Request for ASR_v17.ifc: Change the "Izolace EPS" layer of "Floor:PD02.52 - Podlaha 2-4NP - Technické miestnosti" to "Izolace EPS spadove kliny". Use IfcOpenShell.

First a look at what the model holds.

```python
import ifcopenshell
import ifcopenshell.util.element

model = ifcopenshell.open("ASR_v17.ifc")
print(model.schema)
for layer_set in model.by_type("IfcMaterialLayerSet"):
    if layer_set.LayerSetName == "Floor:PD02.52 - Podlaha 2-4NP - Technické miestnosti":
        for layer in layer_set.MaterialLayers:
            print(layer.id(), layer.Material and layer.Material.Name, layer.LayerThickness, sep=" | ")
        print(len(ifcopenshell.util.element.get_elements_by_material(model, layer_set)), "elements and types use it")
print(sorted(m.Name for m in model.by_type("IfcMaterial") if m.Name)[:60])
```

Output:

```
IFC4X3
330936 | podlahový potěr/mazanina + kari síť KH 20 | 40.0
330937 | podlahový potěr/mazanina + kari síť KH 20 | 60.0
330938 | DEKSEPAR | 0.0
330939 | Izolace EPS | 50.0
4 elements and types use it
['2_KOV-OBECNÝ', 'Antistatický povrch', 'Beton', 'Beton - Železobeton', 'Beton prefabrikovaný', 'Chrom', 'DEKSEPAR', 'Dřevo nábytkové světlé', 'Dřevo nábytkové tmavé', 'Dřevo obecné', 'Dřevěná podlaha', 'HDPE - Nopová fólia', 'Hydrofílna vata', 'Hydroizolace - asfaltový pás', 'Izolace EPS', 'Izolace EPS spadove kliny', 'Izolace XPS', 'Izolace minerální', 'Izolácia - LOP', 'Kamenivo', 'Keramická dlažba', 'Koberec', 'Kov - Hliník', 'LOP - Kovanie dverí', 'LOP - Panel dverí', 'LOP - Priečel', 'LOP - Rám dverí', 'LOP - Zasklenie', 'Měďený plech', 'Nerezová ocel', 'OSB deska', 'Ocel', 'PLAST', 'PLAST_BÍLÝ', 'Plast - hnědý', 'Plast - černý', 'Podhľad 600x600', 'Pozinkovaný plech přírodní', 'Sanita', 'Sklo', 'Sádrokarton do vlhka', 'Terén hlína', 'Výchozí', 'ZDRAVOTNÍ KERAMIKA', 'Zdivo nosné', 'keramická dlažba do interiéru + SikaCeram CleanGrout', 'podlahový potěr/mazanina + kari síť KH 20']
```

```python
import ifcopenshell
import ifcopenshell.api.material

model = ifcopenshell.open("ASR_v17.ifc")

layer_set = next(s for s in model.by_type("IfcMaterialLayerSet") if s.LayerSetName == "Floor:PD02.52 - Podlaha 2-4NP - Technické miestnosti")
layer = next(l for l in layer_set.MaterialLayers if l.Material and l.Material.Name == "Izolace EPS")
material = next(m for m in model.by_type("IfcMaterial") if m.Name == "Izolace EPS spadove kliny")

# Point this one layer at the other material; renaming the old one would change it everywhere.
ifcopenshell.api.material.edit_layer(model, layer=layer, attributes={"Name": material.Name}, material=material)

print([l.Material.Name if l.Material else None for l in layer_set.MaterialLayers])

model.write("ASR_v17-out.ifc")
```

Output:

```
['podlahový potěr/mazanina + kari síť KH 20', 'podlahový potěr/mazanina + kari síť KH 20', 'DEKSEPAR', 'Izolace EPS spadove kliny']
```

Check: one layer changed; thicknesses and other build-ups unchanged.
